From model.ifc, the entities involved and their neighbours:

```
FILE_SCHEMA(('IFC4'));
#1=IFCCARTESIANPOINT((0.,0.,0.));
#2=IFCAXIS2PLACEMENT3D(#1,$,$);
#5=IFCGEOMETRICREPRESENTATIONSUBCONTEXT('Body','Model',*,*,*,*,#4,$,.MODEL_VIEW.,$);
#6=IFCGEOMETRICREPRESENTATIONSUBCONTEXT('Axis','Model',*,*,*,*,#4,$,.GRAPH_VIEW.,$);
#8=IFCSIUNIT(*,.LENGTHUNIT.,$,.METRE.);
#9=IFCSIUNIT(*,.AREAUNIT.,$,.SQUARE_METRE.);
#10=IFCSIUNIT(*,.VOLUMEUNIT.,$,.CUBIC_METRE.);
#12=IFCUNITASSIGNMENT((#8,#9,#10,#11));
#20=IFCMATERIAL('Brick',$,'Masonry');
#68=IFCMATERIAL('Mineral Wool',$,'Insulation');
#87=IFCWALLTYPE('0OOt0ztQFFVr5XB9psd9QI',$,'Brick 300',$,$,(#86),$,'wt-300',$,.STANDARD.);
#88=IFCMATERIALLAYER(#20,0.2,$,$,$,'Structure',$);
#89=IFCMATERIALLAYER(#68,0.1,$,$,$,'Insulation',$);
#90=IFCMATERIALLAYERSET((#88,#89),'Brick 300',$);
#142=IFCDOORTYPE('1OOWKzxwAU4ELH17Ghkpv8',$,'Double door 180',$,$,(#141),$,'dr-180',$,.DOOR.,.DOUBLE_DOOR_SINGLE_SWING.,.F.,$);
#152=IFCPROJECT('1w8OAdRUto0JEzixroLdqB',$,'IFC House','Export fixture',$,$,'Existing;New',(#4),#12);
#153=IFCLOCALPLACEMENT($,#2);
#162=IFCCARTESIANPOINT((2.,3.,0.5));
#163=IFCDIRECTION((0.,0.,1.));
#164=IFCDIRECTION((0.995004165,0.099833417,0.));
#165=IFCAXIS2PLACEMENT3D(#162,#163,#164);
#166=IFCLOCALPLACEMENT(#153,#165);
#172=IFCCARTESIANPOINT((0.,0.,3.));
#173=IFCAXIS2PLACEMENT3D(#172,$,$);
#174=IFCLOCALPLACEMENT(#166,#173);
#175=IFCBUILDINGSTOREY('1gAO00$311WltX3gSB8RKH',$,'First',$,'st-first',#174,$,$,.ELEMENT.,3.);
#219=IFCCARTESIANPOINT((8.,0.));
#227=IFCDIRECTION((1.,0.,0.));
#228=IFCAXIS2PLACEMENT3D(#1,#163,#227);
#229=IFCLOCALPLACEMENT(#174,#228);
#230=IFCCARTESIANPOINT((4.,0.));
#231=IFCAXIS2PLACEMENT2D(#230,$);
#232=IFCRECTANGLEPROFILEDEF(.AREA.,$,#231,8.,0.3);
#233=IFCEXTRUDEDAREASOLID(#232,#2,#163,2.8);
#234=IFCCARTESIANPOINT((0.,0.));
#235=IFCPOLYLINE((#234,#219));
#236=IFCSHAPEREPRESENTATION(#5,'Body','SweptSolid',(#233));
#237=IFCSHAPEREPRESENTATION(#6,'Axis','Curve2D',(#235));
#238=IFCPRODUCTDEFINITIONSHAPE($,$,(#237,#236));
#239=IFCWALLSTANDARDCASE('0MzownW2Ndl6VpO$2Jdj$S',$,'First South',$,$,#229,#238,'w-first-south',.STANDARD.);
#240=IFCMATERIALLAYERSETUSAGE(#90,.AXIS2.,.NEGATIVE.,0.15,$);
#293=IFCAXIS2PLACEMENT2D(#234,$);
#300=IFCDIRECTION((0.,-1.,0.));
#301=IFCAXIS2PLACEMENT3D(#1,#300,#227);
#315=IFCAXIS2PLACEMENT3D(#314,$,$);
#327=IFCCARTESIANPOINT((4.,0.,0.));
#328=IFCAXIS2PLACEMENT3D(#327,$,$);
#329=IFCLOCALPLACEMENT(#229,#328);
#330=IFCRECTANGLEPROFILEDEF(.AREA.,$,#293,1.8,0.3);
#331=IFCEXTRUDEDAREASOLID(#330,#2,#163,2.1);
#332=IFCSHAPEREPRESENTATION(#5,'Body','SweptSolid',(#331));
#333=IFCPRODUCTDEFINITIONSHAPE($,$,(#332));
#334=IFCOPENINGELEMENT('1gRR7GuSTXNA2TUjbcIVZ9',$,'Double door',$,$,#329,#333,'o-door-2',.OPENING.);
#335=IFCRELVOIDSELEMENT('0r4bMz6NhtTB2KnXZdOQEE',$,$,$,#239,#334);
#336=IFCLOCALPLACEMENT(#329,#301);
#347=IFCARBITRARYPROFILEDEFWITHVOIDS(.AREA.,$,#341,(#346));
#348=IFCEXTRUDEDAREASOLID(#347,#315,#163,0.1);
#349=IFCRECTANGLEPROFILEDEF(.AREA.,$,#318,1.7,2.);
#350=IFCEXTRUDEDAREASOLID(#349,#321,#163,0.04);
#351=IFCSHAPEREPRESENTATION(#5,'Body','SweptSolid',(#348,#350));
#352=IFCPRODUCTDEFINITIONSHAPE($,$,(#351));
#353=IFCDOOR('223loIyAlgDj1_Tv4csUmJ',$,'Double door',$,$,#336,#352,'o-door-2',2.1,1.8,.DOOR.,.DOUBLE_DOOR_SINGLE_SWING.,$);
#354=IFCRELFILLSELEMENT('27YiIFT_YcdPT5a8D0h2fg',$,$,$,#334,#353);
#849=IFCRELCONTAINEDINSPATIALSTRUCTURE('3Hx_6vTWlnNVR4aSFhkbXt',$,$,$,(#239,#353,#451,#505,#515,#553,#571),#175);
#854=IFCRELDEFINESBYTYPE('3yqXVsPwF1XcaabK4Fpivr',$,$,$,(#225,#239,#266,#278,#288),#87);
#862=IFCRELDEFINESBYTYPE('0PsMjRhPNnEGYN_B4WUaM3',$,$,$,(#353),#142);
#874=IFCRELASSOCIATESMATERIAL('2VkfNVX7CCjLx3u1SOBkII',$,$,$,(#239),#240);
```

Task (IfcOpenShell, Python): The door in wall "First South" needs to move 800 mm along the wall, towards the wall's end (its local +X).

```python
import ifcopenshell
import ifcopenshell.api.geometry
import ifcopenshell.util.placement

model = ifcopenshell.open("model.ifc")

door = model.by_guid("223loIyAlgDj1_Tv4csUmJ")
opening = door.FillsVoids[0].RelatingOpeningElement
wall = opening.VoidsElements[0].RelatingBuildingElement

wall_matrix = ifcopenshell.util.placement.get_local_placement(wall.ObjectPlacement)
shift = wall_matrix[:3, 0] * 0.8
before = ifcopenshell.util.placement.get_local_placement(door.ObjectPlacement)[:3, 3].copy()

# The door is placed relative to its opening, so it follows when the opening moves.
matrix = ifcopenshell.util.placement.get_local_placement(opening.ObjectPlacement)
matrix[:3, 3] += shift
ifcopenshell.api.geometry.edit_object_placement(
    model, product=opening, matrix=matrix, is_si=False, should_transform_children=True
)

after = ifcopenshell.util.placement.get_local_placement(door.ObjectPlacement)[:3, 3]
print("door moved by", (after - before).round(3) + 0.0)

model.write("model-out.ifc")
```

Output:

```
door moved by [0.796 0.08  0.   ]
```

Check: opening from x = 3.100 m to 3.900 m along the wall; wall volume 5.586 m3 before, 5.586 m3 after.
